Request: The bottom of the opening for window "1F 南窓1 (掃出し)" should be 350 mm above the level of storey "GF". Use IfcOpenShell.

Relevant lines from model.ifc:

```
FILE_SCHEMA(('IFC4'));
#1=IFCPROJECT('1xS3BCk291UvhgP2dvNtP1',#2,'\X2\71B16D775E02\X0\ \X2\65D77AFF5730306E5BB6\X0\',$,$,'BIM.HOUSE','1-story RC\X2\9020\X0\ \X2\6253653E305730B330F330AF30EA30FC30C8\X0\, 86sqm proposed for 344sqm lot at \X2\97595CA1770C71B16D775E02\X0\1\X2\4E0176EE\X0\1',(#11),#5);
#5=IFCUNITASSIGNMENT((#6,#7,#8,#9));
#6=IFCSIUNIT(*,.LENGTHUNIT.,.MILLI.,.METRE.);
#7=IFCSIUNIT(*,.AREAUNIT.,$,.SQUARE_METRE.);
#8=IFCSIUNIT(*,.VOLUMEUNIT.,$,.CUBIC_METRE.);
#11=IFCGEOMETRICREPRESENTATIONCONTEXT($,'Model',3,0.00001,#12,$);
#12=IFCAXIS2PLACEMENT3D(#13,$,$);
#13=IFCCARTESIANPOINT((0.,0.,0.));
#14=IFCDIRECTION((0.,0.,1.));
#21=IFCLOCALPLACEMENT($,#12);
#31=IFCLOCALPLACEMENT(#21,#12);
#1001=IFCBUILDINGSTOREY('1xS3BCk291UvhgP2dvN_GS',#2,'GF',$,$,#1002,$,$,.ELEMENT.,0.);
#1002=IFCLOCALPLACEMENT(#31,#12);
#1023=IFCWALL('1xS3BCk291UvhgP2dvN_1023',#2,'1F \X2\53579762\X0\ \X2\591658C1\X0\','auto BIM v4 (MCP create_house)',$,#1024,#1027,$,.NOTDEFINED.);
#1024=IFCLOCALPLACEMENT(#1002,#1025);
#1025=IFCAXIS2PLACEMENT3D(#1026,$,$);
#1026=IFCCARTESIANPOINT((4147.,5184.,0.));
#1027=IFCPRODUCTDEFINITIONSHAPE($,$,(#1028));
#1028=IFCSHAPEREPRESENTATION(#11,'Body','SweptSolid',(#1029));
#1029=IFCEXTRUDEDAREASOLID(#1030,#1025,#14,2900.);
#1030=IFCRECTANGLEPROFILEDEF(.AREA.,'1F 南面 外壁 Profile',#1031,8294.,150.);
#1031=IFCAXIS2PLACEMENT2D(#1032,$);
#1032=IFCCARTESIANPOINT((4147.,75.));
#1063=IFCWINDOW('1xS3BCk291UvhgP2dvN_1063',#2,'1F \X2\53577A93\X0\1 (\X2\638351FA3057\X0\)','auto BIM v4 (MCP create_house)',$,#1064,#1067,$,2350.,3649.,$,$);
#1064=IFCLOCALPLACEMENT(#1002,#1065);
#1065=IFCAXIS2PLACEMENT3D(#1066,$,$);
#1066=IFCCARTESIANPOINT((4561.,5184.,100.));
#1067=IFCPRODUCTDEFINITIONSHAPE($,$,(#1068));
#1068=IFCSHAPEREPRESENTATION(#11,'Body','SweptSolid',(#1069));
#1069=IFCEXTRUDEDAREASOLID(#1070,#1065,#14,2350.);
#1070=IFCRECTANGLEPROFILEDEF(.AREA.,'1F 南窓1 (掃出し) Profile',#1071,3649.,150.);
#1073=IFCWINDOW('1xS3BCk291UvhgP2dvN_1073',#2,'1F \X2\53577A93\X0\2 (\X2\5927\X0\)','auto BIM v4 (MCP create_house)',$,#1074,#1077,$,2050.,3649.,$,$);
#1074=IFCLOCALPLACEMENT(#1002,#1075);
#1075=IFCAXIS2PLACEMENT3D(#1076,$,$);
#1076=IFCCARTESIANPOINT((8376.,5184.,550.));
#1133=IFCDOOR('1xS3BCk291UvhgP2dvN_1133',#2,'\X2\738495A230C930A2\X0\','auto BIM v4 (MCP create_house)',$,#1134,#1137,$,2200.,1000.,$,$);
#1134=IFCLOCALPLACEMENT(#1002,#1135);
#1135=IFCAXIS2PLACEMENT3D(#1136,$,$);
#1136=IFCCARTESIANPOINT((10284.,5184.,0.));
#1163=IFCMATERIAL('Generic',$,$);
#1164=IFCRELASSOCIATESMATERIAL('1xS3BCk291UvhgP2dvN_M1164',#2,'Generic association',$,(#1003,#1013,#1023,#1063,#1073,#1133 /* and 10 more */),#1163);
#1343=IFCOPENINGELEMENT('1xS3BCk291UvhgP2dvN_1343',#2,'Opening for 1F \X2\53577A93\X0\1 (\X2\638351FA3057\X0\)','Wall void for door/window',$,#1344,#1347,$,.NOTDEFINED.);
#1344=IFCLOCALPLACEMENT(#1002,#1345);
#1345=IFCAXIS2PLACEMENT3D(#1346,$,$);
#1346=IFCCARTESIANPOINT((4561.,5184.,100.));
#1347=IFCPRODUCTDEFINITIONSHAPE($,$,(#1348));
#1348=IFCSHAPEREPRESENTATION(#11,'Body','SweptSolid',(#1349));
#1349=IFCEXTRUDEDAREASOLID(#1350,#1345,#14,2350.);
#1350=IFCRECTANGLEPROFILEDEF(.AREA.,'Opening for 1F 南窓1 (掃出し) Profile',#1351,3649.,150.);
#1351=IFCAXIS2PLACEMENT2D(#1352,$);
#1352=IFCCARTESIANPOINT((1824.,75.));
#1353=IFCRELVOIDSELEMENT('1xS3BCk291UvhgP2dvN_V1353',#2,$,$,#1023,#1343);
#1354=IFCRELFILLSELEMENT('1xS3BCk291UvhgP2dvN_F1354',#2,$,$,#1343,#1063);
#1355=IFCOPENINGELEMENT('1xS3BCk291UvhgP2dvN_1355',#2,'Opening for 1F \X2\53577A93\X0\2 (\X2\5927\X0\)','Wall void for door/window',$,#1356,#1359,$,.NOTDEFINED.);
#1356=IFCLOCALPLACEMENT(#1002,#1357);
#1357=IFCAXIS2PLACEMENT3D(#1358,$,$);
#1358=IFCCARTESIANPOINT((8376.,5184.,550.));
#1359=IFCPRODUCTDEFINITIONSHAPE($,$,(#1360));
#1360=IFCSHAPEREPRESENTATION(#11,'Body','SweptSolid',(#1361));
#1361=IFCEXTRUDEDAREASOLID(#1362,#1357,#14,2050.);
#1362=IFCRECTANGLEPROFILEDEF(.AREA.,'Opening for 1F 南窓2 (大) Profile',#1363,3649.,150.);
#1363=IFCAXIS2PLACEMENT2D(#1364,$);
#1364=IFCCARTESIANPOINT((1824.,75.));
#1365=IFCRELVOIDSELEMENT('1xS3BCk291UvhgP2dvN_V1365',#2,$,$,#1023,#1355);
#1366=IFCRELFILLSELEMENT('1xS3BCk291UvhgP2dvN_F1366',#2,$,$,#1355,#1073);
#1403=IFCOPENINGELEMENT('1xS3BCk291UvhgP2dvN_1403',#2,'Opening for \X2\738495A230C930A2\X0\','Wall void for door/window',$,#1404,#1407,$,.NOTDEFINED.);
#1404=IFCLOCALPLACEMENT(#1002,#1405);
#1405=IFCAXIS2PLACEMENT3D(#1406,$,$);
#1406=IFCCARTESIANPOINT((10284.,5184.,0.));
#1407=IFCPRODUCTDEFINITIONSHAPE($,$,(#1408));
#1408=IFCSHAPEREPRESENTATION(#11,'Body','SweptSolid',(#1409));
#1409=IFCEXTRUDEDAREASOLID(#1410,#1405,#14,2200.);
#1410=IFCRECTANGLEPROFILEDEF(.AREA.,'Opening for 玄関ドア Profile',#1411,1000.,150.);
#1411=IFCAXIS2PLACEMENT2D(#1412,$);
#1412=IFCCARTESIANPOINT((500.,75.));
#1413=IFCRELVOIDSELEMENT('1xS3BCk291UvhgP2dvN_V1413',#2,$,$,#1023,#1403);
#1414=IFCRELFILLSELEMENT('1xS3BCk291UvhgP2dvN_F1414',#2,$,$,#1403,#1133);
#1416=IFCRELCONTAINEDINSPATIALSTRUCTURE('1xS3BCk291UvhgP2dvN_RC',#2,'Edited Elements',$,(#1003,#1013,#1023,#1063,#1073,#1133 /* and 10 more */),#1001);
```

```python
import numpy as np
import ifcopenshell
import ifcopenshell.api.geometry
import ifcopenshell.geom
import ifcopenshell.util.element
import ifcopenshell.util.placement
import ifcopenshell.util.shape
import ifcopenshell.util.unit

model = ifcopenshell.open("model.ifc")
unit_scale = ifcopenshell.util.unit.calculate_unit_scale(model)

window = model.by_guid("1xS3BCk291UvhgP2dvN_1063")
opening = window.FillsVoids[0].RelatingOpeningElement
storey = ifcopenshell.util.element.get_container(window, ifc_class="IfcBuildingStorey")
level = ifcopenshell.util.placement.get_local_placement(storey.ObjectPlacement)[2, 3]

# The opening's origin need not be at the sill, so measure its lowest point.
shape = ifcopenshell.geom.create_shape(ifcopenshell.geom.settings(), opening)
bottom = ifcopenshell.util.shape.get_shape_bottom_elevation(shape, shape.geometry) / unit_scale
dz = level + 350.0 - bottom

shift = np.array([0.0, 0.0, dz])
# The window is not placed relative to its opening, so move both.
for product in (opening, window):
    matrix = ifcopenshell.util.placement.get_local_placement(product.ObjectPlacement)
    matrix[:3, 3] += shift
    ifcopenshell.api.geometry.edit_object_placement(model, product=product, matrix=matrix, is_si=False)

print(f"moved by {dz * unit_scale:+.3f} m")

model.write("model_updated.ifc")
```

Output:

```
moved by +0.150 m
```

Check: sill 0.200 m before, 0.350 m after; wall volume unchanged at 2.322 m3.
